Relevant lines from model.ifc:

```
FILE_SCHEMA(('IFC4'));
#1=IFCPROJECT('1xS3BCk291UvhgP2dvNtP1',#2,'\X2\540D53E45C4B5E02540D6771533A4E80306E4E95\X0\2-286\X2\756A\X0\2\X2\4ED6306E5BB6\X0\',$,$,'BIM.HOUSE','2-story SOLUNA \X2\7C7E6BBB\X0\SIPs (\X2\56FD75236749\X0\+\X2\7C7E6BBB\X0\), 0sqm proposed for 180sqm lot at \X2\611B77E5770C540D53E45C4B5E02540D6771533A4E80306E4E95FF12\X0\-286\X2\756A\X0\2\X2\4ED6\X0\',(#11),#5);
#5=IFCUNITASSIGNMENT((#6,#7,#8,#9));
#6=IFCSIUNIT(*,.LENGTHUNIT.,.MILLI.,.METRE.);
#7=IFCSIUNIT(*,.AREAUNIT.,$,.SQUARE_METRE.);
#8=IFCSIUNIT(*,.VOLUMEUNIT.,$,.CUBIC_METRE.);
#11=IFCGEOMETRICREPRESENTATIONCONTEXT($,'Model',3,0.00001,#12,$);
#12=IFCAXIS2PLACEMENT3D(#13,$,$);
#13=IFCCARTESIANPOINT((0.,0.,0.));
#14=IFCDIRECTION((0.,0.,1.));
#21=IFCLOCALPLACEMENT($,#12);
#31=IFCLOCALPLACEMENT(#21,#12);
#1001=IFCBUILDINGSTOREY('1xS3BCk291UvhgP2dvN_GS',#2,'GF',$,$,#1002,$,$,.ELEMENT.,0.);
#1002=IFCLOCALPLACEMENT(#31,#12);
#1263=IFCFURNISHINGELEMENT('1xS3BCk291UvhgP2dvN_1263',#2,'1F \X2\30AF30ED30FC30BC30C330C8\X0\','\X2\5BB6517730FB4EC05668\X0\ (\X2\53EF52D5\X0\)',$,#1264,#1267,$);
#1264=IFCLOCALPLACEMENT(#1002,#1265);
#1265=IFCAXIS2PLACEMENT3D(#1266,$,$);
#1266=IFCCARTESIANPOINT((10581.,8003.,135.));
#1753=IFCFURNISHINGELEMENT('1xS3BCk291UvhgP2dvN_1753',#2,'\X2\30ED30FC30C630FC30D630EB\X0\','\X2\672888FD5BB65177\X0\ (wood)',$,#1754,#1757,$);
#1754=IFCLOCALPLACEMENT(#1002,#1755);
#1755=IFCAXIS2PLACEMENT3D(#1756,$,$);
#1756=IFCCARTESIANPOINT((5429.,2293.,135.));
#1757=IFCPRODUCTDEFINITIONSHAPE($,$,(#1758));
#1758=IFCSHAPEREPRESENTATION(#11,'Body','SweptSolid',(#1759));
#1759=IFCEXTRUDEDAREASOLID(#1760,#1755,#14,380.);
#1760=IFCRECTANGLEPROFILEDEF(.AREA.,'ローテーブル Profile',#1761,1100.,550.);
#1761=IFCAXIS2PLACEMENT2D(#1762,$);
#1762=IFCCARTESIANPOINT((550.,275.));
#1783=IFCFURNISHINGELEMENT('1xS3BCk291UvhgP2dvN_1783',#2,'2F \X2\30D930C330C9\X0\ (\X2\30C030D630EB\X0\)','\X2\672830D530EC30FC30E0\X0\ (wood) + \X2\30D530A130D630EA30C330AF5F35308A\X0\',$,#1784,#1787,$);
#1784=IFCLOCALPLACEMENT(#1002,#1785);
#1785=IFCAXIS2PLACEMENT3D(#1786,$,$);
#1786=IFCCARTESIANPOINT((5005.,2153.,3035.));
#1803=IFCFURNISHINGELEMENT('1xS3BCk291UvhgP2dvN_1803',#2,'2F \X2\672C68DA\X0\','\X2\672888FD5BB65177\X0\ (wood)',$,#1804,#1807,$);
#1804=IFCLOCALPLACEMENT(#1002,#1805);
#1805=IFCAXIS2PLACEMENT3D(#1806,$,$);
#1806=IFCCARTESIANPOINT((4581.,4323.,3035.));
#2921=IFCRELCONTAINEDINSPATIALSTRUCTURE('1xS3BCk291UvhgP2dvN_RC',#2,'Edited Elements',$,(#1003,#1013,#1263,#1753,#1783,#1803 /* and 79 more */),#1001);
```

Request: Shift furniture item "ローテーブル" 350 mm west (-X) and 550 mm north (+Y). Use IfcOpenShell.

```python
import ifcopenshell
import ifcopenshell.api.geometry
import ifcopenshell.util.placement

model = ifcopenshell.open("model.ifc")

item = model.by_guid("1xS3BCk291UvhgP2dvN_1753")
matrix = ifcopenshell.util.placement.get_local_placement(item.ObjectPlacement)
matrix[0, 3] -= 350.0
matrix[1, 3] += 550.0
ifcopenshell.api.geometry.edit_object_placement(model, product=item, matrix=matrix, is_si=False)

print(ifcopenshell.util.placement.get_local_placement(item.ObjectPlacement).round(3) + 0.0)

model.write("model-out.ifc")
```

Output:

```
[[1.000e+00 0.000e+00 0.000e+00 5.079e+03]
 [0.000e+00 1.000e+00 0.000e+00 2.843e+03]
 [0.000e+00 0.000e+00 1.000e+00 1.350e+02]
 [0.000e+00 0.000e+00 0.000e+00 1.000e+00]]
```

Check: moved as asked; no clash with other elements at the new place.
